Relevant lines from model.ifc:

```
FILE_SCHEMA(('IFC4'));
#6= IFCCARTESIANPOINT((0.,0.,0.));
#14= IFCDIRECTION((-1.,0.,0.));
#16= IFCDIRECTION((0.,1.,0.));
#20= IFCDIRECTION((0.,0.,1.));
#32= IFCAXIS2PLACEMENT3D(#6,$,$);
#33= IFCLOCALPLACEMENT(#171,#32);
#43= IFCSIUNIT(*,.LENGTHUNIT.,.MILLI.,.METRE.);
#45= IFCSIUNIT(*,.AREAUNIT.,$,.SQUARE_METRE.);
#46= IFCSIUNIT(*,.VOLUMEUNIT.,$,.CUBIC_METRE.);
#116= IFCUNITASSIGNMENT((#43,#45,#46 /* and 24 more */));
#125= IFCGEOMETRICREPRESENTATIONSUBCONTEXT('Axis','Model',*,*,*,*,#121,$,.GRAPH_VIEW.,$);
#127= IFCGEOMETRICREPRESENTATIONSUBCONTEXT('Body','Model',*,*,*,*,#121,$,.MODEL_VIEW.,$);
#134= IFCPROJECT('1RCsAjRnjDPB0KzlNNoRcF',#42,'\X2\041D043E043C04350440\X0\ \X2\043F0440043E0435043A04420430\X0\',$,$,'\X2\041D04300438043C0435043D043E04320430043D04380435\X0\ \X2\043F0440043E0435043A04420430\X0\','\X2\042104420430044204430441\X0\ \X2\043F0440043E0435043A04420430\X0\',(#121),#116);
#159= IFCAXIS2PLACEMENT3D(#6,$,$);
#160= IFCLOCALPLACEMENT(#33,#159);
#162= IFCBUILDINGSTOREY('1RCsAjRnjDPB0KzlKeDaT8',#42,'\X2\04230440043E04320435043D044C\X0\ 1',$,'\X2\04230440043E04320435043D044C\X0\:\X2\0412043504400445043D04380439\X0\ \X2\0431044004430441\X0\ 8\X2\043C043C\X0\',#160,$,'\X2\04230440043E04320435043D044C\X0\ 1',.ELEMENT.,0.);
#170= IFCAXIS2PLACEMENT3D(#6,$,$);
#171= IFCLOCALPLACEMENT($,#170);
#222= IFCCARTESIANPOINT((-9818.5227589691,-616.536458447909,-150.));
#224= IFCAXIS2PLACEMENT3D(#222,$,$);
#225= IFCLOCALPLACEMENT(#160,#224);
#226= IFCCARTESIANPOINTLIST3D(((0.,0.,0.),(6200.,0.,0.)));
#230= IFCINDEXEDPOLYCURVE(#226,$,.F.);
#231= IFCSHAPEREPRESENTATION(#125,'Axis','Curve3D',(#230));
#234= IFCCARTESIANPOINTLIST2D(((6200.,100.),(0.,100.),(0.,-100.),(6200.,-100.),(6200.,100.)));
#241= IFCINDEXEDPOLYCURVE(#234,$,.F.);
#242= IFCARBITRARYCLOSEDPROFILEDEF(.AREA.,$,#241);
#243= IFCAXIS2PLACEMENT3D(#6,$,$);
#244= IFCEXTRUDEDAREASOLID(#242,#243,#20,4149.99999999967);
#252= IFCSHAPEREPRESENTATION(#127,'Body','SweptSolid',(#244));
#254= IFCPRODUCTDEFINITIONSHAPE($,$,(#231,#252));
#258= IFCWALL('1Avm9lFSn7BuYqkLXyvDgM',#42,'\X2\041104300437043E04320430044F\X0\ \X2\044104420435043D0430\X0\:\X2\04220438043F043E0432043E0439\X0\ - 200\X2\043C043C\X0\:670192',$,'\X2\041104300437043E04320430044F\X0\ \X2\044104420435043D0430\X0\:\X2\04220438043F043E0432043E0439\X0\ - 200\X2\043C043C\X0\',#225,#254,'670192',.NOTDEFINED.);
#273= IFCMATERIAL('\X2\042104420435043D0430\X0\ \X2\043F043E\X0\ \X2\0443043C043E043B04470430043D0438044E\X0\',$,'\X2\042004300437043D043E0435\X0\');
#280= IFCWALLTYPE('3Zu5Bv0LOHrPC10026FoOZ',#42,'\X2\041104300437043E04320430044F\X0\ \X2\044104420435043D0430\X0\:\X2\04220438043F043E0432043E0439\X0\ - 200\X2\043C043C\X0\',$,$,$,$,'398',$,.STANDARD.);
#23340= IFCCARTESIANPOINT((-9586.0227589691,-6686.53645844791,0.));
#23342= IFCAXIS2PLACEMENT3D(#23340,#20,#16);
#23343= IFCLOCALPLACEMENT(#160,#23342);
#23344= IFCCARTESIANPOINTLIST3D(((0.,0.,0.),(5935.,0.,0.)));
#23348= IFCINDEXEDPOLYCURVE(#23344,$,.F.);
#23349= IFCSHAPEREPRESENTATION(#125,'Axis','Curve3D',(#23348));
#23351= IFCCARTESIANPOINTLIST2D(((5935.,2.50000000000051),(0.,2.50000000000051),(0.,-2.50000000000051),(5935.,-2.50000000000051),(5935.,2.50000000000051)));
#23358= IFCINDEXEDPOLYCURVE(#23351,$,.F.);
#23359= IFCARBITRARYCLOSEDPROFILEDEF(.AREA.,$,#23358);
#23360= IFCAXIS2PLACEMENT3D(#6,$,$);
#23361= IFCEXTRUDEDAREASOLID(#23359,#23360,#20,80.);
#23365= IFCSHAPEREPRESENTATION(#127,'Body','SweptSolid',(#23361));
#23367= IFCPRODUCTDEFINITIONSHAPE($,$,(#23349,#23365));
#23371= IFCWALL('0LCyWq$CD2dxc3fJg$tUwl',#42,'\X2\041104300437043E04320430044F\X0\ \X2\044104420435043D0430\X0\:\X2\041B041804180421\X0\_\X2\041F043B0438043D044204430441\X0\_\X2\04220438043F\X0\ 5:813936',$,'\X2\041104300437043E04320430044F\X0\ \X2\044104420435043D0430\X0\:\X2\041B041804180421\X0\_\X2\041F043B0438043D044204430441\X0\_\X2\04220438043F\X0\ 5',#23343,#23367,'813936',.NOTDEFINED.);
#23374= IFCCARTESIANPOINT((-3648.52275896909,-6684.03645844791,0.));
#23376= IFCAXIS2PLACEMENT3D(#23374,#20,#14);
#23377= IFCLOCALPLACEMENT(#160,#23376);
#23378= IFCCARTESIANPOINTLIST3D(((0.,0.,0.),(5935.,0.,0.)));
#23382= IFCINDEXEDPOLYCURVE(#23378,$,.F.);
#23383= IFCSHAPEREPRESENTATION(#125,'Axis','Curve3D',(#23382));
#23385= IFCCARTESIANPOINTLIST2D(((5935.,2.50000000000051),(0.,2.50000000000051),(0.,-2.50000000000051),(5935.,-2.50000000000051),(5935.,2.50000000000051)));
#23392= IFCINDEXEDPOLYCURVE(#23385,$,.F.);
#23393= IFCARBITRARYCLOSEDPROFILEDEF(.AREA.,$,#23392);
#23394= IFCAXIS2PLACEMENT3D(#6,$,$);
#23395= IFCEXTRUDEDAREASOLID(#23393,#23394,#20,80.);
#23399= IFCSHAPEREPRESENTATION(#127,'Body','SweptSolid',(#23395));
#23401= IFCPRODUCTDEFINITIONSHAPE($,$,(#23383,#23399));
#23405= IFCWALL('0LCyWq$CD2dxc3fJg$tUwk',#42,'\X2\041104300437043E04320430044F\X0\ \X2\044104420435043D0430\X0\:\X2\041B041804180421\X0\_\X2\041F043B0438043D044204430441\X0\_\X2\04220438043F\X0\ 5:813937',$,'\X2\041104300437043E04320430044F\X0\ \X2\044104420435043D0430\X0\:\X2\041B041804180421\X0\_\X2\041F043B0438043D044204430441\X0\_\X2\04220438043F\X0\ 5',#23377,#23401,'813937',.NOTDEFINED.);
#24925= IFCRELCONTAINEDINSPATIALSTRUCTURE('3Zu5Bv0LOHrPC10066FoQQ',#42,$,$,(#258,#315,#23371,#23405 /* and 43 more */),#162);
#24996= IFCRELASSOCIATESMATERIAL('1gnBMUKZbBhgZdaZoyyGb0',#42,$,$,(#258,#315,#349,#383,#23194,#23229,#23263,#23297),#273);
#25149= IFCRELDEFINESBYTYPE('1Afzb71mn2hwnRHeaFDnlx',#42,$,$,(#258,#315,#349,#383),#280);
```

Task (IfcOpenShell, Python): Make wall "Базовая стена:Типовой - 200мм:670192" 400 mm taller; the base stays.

```python
import ifcopenshell
import ifcopenshell.geom
import ifcopenshell.util.representation
import ifcopenshell.util.shape

model = ifcopenshell.open("model.ifc")
settings = ifcopenshell.geom.settings()


def volume(element):
    """Net volume in cubic metres, openings subtracted."""
    shape = ifcopenshell.geom.create_shape(settings, element)
    return ifcopenshell.util.shape.get_volume(shape.geometry)


wall = model.by_guid("1Avm9lFSn7BuYqkLXyvDgM")
before = volume(wall)

body = ifcopenshell.util.representation.get_representation(wall, "Model", "Body")
solid = body.Items[0]
old_height = solid.Depth
solid.Depth += 400.0
after = volume(wall)

print(f"height {old_height:g} -> {solid.Depth:g}, volume {before:.3f} -> {after:.3f} m3")

model.write("model_updated.ifc")
```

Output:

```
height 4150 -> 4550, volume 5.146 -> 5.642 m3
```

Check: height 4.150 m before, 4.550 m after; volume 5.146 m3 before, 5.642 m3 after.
